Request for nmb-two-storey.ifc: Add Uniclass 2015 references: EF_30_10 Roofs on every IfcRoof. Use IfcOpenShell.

First a look at what the model holds.

```python
import ifcopenshell

model = ifcopenshell.open("nmb-two-storey.ifc")
print(model.schema)
print("classifications:", [c.Name for c in model.by_type("IfcClassification")])
for ifc_class in ("IfcDoor", "IfcRoof", "IfcStair", "IfcWall", "IfcWindow"):
    print(ifc_class, len(model.by_type(ifc_class)))
```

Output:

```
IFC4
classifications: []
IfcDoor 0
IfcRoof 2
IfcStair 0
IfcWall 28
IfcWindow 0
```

```python
import ifcopenshell
import ifcopenshell.api.classification

model = ifcopenshell.open("nmb-two-storey.ifc")

system = ifcopenshell.api.classification.add_classification(model, classification="Uniclass 2015")

codes = {
    "IfcRoof": ("EF_30_10", "Roofs"),
}
for ifc_class, (code, name) in codes.items():
    products = model.by_type(ifc_class)
    ifcopenshell.api.classification.add_reference(
        model, products=products, classification=system, identification=code, name=name
    )
    print(code, len(products))

model.write("nmb-two-storey-out.ifc")
```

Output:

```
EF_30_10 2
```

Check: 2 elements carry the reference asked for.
